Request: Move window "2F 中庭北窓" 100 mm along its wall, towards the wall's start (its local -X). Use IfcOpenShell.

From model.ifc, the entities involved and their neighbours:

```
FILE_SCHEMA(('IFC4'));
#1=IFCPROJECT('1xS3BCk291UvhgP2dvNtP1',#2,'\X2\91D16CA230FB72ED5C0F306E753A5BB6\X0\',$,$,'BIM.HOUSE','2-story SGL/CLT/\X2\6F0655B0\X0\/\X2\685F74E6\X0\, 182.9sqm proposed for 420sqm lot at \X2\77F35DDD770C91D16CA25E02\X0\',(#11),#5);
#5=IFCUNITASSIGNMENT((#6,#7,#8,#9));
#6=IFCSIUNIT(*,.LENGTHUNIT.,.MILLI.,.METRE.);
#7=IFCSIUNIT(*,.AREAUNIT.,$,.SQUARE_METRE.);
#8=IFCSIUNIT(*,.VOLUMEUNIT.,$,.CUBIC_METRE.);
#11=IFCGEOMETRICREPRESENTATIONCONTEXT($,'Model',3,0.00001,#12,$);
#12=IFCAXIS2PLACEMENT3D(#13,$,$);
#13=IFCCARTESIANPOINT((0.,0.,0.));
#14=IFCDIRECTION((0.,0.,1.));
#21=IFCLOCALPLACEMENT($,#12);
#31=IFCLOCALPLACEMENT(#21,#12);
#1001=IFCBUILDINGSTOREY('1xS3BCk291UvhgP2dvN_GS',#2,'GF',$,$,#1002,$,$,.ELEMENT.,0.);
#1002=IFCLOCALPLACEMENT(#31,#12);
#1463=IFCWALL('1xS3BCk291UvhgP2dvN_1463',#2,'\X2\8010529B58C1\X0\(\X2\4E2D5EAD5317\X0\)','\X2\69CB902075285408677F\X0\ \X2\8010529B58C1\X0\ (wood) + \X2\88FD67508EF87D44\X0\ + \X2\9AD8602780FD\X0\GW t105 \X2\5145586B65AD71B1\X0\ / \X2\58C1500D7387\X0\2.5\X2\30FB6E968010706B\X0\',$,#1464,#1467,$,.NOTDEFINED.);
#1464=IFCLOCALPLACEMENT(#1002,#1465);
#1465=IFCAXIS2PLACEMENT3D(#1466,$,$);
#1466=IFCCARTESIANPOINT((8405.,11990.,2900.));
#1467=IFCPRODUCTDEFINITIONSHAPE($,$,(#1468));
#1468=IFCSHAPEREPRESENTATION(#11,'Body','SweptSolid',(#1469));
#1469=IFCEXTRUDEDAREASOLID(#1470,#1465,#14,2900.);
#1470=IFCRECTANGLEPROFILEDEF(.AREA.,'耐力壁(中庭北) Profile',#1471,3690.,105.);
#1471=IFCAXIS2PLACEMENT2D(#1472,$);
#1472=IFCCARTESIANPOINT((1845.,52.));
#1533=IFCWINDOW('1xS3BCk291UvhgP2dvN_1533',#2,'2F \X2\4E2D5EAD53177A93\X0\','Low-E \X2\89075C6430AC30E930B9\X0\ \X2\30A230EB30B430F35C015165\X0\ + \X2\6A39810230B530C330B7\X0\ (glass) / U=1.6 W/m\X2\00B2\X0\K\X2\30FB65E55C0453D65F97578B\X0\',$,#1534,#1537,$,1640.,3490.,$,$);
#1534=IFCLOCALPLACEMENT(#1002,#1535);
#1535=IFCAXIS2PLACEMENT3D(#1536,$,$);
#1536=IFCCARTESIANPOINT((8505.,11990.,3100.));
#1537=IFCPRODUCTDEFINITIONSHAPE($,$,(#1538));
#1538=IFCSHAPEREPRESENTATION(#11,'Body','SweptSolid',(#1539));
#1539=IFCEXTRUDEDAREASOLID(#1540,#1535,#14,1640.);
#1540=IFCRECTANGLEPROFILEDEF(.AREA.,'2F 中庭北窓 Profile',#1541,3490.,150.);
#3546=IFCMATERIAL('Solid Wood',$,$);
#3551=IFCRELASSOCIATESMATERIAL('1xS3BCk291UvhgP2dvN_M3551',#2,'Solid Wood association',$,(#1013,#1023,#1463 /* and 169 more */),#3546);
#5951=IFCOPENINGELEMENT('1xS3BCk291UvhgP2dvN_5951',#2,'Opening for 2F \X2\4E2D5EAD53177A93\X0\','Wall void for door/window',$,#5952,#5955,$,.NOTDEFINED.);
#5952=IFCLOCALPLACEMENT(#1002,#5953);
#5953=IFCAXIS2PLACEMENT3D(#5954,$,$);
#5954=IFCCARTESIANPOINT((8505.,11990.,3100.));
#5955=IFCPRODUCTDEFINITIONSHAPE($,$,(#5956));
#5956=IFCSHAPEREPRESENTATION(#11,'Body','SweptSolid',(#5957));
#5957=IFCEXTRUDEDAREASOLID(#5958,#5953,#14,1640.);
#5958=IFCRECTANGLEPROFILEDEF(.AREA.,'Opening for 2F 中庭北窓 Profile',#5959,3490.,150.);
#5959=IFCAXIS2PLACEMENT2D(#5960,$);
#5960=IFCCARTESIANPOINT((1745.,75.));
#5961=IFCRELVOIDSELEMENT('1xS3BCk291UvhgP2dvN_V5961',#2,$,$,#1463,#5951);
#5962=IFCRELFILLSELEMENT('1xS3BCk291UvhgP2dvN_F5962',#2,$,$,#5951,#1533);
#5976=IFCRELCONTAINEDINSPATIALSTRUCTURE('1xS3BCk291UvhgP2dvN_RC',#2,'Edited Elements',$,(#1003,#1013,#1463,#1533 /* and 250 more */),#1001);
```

```python
import ifcopenshell
import ifcopenshell.api.geometry
import ifcopenshell.util.placement
import ifcopenshell.util.unit

model = ifcopenshell.open("model.ifc")
unit_scale = ifcopenshell.util.unit.calculate_unit_scale(model)

window = model.by_id(1533)
opening = window.FillsVoids[0].RelatingOpeningElement
wall = opening.VoidsElements[0].RelatingBuildingElement

wall_matrix = ifcopenshell.util.placement.get_local_placement(wall.ObjectPlacement)
shift = wall_matrix[:3, 0] * -0.1 / unit_scale
before = ifcopenshell.util.placement.get_local_placement(window.ObjectPlacement)[:3, 3].copy()

# The window is not placed relative to its opening, so move both.
for product in (opening, window):
    matrix = ifcopenshell.util.placement.get_local_placement(product.ObjectPlacement)
    matrix[:3, 3] += shift
    ifcopenshell.api.geometry.edit_object_placement(model, product=product, matrix=matrix, is_si=False)

after = ifcopenshell.util.placement.get_local_placement(window.ObjectPlacement)[:3, 3]
print("window moved by", (after - before).round(3) + 0.0)

model.write("model_v2.ifc")
```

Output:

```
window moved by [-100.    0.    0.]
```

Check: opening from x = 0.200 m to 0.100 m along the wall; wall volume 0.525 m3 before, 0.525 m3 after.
